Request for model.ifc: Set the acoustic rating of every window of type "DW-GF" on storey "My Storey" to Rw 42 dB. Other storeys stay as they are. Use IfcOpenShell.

First a look at what the model holds.

```python
import ifcopenshell
import ifcopenshell.util.element

model = ifcopenshell.open("model.ifc")
print(model.schema)
storey = next(s for s in model.by_type("IfcBuildingStorey") if s.Name == "My Storey")
windows = [e for e in ifcopenshell.util.element.get_decomposition(storey) if e.is_a("IfcWindow")]
seen = {}
for e in windows:
    element_type = ifcopenshell.util.element.get_type(e)
    key = (element_type.Name if element_type != e and element_type else None, ifcopenshell.util.element.get_pset(e, "Pset_WindowCommon", "AcousticRating"))
    seen[key] = seen.get(key, 0) + 1
for (name, value), count in sorted(seen.items(), key=str):
    print(count, "x", name, "|", value)
```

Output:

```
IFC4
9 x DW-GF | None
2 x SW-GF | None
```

```python
import ifcopenshell
import ifcopenshell.api.pset
import ifcopenshell.util.element

model = ifcopenshell.open("model.ifc")

storey = next(s for s in model.by_type("IfcBuildingStorey") if s.Name == "My Storey")
windows = [e for e in ifcopenshell.util.element.get_decomposition(storey) if e.is_a("IfcWindow")]

count = 0
for e in windows:
    element_type = ifcopenshell.util.element.get_type(e)
    if element_type in (None, e) or element_type.Name != "DW-GF":
        continue
    # add_pset returns the element's existing set when there is one.
    pset = ifcopenshell.api.pset.add_pset(model, product=e, name="Pset_WindowCommon")
    ifcopenshell.api.pset.edit_pset(model, pset=pset, properties={"AcousticRating": "Rw 42 dB"})
    count += 1

print(count, "windows updated")

model.write("model_v2.ifc")
```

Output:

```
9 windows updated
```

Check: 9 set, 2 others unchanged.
